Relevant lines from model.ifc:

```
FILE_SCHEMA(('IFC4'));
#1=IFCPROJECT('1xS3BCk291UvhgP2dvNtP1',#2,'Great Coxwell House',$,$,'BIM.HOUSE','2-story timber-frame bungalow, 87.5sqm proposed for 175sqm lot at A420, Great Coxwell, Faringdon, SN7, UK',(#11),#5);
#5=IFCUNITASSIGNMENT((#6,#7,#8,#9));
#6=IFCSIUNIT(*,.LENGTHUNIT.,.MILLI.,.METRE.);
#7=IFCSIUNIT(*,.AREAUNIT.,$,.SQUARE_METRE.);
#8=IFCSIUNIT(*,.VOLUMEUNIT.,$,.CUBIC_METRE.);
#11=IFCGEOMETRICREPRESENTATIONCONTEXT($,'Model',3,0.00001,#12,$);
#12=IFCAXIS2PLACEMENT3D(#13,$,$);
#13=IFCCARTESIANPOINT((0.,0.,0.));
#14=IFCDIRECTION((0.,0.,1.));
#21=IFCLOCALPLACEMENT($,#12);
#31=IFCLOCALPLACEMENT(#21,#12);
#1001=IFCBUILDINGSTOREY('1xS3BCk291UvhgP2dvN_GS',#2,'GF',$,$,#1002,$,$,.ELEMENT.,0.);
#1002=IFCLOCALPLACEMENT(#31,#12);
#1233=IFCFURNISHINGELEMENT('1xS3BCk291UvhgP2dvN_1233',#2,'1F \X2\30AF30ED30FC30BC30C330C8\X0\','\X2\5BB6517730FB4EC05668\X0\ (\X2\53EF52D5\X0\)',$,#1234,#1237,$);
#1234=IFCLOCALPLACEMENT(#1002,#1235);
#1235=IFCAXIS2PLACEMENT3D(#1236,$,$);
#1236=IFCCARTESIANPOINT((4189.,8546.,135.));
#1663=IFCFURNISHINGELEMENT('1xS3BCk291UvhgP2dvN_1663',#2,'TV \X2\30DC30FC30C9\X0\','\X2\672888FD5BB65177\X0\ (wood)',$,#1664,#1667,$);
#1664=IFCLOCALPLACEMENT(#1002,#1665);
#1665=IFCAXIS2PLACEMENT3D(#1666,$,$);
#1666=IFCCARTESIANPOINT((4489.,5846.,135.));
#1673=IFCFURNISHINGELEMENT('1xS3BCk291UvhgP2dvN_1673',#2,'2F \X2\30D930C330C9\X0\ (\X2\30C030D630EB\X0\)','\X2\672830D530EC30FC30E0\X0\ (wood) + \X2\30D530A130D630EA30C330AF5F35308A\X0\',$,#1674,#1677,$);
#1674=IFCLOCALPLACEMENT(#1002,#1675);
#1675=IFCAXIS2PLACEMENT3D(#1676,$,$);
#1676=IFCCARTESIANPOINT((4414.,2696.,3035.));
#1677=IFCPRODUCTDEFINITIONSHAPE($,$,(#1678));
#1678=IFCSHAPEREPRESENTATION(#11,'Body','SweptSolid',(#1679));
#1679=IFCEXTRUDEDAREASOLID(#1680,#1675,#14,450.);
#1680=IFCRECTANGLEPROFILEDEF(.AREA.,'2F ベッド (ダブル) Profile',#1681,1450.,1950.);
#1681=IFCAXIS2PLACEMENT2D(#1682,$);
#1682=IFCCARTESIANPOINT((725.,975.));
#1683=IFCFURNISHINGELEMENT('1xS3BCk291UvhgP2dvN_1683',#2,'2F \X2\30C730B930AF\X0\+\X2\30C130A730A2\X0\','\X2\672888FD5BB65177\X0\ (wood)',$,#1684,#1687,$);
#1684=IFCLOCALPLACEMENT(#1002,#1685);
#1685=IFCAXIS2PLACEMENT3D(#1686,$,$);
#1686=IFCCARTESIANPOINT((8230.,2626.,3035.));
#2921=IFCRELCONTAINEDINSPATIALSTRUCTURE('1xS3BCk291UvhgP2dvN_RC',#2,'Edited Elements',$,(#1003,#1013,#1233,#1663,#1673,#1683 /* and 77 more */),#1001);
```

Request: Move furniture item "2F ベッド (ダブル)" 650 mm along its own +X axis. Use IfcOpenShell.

```python
import ifcopenshell
import ifcopenshell.api.geometry
import ifcopenshell.util.placement

model = ifcopenshell.open("model.ifc")

item = model.by_guid("1xS3BCk291UvhgP2dvN_1673")
matrix = ifcopenshell.util.placement.get_local_placement(item.ObjectPlacement)
matrix[:3, 3] += matrix[:3, 0] * 650.0
ifcopenshell.api.geometry.edit_object_placement(model, product=item, matrix=matrix, is_si=False)

print(ifcopenshell.util.placement.get_local_placement(item.ObjectPlacement).round(3) + 0.0)

model.write("model_rev.ifc")
```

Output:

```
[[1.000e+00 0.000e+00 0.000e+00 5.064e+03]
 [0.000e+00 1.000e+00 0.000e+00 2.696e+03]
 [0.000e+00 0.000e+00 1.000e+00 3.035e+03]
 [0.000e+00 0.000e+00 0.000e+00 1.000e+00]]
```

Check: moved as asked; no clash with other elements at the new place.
